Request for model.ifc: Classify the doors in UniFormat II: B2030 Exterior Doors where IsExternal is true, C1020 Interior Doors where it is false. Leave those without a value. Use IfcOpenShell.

First a look at what the model holds.

```python
import ifcopenshell
import ifcopenshell.util.element

model = ifcopenshell.open("model.ifc")
print(model.schema)
print("classifications:", [c.Name for c in model.by_type("IfcClassification")])
values = [ifcopenshell.util.element.get_pset(e, "Pset_DoorCommon", "IsExternal") for e in model.by_type("IfcDoor")]
for value in (True, False, None):
    print("IsExternal", value, values.count(value))
```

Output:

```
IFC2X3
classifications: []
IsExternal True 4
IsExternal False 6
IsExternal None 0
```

```python
import ifcopenshell
import ifcopenshell.api.classification
import ifcopenshell.util.element

model = ifcopenshell.open("model.ifc")

# IFC2X3 requires Source and Edition and has no link from the project to the system.
system = model.create_entity("IfcClassification", Source="ASTM", Edition="E1557", Name="UniFormat II")

doors = model.by_type("IfcDoor")
external = {e: ifcopenshell.util.element.get_pset(e, "Pset_DoorCommon", "IsExternal") for e in doors}
for flag, code, name in ((True, "B2030", "Exterior Doors"), (False, "C1020", "Interior Doors")):
    products = [e for e in doors if external[e] is flag]
    ifcopenshell.api.classification.add_reference(
        model, products=products, classification=system, identification=code, name=name
    )
    print(code, len(products))

model.write("model_updated.ifc")
```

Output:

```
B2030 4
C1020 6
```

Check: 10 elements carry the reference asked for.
